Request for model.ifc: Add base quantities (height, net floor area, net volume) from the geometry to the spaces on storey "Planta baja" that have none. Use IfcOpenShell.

First a look at what the model holds.

```python
import ifcopenshell
import ifcopenshell.util.element
import ifcopenshell.util.unit

model = ifcopenshell.open("model.ifc")
print(model.schema)
for unit_type in ("LENGTHUNIT", "AREAUNIT", "VOLUMEUNIT"):
    print(unit_type, ifcopenshell.util.unit.calculate_unit_scale(model, unit_type))
storey = next(s for s in model.by_type("IfcBuildingStorey") if s.Name == "Planta baja")
spaces = [e for e in ifcopenshell.util.element.get_decomposition(storey) if e.is_a("IfcSpace")]
for e in sorted(spaces, key=lambda e: e.id()):
    print(e.id(), e.is_a(), e.Name, list(ifcopenshell.util.element.get_psets(e, qtos_only=True)), sep=" | ")
```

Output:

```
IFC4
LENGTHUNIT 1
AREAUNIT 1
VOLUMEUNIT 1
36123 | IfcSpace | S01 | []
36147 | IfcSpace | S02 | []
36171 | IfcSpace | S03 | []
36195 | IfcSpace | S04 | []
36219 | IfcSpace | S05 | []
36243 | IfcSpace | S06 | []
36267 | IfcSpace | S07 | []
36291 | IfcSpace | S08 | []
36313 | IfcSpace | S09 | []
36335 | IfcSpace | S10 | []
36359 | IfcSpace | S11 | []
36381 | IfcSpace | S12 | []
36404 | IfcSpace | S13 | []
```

```python
import ifcopenshell
import ifcopenshell.api.pset
import ifcopenshell.geom
import ifcopenshell.util.element
import ifcopenshell.util.shape
import ifcopenshell.util.unit

model = ifcopenshell.open("model.ifc")
unit_scale = ifcopenshell.util.unit.calculate_unit_scale(model)
area_scale = ifcopenshell.util.unit.calculate_unit_scale(model, "AREAUNIT")
volume_scale = ifcopenshell.util.unit.calculate_unit_scale(model, "VOLUMEUNIT")
settings = ifcopenshell.geom.settings()

storey = next(s for s in model.by_type("IfcBuildingStorey") if s.Name == "Planta baja")
spaces = [e for e in ifcopenshell.util.element.get_decomposition(storey) if e.is_a("IfcSpace")]

for e in sorted(spaces, key=lambda e: e.id()):
    if ifcopenshell.util.element.get_psets(e, qtos_only=True, should_inherit=False):
        continue
    # Geometry comes back in metres, in the element's own axes.
    shape = ifcopenshell.geom.create_shape(settings, e)
    values = {
        "Height": ifcopenshell.util.shape.get_z(shape.geometry) / unit_scale,
        "NetFloorArea": ifcopenshell.util.shape.get_footprint_area(shape.geometry) / area_scale,
        "NetVolume": ifcopenshell.util.shape.get_volume(shape.geometry) / volume_scale,
    }
    qto = ifcopenshell.api.pset.add_qto(model, product=e, name="Qto_SpaceBaseQuantities")
    ifcopenshell.api.pset.edit_qto(model, qto=qto, properties=values)
    print(e.id(), {k: round(v, 3) for k, v in values.items()})

model.write("model_edited.ifc")
```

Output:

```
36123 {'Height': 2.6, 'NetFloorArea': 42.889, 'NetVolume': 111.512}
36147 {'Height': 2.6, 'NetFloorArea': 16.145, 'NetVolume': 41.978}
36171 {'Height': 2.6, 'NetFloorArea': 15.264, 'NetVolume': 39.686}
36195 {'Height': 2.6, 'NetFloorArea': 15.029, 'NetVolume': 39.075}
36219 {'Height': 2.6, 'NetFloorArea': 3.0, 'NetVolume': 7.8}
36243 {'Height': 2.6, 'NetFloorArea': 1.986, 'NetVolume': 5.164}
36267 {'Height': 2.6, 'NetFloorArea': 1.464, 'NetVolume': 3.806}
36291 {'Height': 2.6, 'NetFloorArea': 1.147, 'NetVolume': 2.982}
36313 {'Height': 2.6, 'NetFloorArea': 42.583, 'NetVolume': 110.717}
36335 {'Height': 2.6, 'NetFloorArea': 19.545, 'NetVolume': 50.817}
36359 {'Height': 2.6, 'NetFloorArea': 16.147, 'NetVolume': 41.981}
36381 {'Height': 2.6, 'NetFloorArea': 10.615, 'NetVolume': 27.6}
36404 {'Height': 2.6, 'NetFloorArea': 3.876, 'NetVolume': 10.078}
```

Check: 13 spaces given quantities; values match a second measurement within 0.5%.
